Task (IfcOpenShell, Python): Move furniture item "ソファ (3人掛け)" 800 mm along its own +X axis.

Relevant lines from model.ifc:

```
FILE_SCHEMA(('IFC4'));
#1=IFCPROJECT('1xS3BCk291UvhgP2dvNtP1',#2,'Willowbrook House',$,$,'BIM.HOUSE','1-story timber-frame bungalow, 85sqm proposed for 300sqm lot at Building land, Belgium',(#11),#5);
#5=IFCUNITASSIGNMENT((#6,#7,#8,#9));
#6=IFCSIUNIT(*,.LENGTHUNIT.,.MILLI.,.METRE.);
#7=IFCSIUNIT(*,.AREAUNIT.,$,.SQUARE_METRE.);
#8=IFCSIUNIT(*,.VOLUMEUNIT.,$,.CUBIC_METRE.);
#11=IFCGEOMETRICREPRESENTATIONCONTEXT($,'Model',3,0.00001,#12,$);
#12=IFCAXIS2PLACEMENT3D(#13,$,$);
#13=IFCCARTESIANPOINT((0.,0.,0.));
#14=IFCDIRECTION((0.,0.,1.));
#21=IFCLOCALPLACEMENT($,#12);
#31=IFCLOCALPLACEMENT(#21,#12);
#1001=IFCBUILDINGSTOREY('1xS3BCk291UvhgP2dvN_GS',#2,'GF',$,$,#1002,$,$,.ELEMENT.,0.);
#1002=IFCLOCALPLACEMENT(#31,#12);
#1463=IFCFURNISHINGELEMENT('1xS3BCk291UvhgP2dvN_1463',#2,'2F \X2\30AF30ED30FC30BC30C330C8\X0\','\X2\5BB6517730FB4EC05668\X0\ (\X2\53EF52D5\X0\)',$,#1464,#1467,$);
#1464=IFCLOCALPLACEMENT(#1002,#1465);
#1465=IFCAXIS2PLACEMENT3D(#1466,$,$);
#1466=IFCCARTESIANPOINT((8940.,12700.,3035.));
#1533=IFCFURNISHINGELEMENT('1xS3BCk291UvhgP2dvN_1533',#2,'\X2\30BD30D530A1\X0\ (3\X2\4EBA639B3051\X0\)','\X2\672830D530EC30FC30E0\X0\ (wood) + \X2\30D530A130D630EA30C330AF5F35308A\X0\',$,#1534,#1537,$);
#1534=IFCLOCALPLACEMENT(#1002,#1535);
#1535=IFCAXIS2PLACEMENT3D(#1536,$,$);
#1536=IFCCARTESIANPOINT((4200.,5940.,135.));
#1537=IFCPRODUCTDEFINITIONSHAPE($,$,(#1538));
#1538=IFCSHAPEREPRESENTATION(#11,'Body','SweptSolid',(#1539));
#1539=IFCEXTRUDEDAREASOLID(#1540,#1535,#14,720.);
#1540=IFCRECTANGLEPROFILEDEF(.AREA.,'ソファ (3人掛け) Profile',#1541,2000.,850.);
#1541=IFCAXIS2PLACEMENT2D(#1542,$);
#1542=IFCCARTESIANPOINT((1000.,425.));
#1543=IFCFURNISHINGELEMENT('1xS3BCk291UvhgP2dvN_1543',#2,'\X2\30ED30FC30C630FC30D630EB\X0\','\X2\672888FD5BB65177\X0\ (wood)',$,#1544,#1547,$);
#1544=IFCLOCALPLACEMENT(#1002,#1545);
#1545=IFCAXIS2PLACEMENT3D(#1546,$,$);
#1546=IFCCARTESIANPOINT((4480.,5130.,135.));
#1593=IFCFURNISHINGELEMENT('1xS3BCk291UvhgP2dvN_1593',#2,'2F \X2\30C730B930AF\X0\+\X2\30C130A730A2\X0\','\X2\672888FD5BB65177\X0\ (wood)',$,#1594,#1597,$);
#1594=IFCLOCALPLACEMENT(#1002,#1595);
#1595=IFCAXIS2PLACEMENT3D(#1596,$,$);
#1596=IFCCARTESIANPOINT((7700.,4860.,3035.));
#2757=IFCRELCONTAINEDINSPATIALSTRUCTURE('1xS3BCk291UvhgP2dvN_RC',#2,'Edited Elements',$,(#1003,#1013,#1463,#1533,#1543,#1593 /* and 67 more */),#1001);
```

```python
import ifcopenshell
import ifcopenshell.api.geometry
import ifcopenshell.util.placement
import ifcopenshell.util.unit

model = ifcopenshell.open("model.ifc")
unit_scale = ifcopenshell.util.unit.calculate_unit_scale(model)

item = model.by_id(1533)
matrix = ifcopenshell.util.placement.get_local_placement(item.ObjectPlacement)
matrix[:3, 3] += matrix[:3, 0] * 0.8 / unit_scale
ifcopenshell.api.geometry.edit_object_placement(model, product=item, matrix=matrix, is_si=False)

print(ifcopenshell.util.placement.get_local_placement(item.ObjectPlacement).round(3) + 0.0)

model.write("model-out.ifc")
```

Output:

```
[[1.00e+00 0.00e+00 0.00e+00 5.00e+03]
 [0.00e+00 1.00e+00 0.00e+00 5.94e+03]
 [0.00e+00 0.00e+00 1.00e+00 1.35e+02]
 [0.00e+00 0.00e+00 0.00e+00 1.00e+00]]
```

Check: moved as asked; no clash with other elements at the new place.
